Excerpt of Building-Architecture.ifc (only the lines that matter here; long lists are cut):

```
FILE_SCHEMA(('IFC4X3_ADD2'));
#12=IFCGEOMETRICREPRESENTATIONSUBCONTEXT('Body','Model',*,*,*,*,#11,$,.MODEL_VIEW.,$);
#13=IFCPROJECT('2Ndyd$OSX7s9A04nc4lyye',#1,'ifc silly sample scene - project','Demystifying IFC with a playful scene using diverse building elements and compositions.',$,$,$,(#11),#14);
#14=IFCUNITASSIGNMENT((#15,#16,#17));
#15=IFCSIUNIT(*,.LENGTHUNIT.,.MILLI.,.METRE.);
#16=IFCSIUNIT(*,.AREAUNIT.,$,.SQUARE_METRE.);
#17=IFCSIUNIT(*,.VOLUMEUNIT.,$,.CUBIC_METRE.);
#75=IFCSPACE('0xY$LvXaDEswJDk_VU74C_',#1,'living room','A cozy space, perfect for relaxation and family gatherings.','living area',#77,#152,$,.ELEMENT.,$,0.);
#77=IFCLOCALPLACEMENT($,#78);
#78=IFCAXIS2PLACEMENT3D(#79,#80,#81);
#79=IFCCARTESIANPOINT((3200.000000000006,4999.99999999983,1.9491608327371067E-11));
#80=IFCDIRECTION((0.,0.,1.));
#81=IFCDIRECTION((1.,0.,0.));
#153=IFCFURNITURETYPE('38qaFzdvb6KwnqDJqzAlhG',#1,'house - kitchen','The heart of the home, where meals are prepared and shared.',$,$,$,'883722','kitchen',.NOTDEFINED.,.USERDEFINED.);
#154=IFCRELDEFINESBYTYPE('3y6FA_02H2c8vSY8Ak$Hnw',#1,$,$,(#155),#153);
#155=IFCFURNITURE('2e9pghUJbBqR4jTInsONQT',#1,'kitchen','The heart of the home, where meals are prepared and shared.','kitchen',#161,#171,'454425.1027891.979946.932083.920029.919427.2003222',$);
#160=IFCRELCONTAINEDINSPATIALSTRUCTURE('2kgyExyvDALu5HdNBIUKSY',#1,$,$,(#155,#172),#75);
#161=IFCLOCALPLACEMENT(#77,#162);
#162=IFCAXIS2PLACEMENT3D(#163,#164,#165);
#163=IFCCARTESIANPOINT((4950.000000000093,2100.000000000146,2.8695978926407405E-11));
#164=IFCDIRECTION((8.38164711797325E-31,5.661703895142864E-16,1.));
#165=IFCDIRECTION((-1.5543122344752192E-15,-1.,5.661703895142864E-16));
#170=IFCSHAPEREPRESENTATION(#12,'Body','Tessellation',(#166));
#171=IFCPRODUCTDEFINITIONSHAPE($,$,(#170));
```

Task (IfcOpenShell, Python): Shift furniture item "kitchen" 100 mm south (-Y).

```python
import ifcopenshell
import ifcopenshell.api.geometry
import ifcopenshell.util.placement
import ifcopenshell.util.unit

model = ifcopenshell.open("Building-Architecture.ifc")
unit_scale = ifcopenshell.util.unit.calculate_unit_scale(model)

item = model.by_guid("2e9pghUJbBqR4jTInsONQT")
matrix = ifcopenshell.util.placement.get_local_placement(item.ObjectPlacement)
matrix[1, 3] -= 0.1 / unit_scale
ifcopenshell.api.geometry.edit_object_placement(model, product=item, matrix=matrix, is_si=False)

print(ifcopenshell.util.placement.get_local_placement(item.ObjectPlacement).round(3) + 0.0)

model.write("Building-Architecture-out.ifc")
```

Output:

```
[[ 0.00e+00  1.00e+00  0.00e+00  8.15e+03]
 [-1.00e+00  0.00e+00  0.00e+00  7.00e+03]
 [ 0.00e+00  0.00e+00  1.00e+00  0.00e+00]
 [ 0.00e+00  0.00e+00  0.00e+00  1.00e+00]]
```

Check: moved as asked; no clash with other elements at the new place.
